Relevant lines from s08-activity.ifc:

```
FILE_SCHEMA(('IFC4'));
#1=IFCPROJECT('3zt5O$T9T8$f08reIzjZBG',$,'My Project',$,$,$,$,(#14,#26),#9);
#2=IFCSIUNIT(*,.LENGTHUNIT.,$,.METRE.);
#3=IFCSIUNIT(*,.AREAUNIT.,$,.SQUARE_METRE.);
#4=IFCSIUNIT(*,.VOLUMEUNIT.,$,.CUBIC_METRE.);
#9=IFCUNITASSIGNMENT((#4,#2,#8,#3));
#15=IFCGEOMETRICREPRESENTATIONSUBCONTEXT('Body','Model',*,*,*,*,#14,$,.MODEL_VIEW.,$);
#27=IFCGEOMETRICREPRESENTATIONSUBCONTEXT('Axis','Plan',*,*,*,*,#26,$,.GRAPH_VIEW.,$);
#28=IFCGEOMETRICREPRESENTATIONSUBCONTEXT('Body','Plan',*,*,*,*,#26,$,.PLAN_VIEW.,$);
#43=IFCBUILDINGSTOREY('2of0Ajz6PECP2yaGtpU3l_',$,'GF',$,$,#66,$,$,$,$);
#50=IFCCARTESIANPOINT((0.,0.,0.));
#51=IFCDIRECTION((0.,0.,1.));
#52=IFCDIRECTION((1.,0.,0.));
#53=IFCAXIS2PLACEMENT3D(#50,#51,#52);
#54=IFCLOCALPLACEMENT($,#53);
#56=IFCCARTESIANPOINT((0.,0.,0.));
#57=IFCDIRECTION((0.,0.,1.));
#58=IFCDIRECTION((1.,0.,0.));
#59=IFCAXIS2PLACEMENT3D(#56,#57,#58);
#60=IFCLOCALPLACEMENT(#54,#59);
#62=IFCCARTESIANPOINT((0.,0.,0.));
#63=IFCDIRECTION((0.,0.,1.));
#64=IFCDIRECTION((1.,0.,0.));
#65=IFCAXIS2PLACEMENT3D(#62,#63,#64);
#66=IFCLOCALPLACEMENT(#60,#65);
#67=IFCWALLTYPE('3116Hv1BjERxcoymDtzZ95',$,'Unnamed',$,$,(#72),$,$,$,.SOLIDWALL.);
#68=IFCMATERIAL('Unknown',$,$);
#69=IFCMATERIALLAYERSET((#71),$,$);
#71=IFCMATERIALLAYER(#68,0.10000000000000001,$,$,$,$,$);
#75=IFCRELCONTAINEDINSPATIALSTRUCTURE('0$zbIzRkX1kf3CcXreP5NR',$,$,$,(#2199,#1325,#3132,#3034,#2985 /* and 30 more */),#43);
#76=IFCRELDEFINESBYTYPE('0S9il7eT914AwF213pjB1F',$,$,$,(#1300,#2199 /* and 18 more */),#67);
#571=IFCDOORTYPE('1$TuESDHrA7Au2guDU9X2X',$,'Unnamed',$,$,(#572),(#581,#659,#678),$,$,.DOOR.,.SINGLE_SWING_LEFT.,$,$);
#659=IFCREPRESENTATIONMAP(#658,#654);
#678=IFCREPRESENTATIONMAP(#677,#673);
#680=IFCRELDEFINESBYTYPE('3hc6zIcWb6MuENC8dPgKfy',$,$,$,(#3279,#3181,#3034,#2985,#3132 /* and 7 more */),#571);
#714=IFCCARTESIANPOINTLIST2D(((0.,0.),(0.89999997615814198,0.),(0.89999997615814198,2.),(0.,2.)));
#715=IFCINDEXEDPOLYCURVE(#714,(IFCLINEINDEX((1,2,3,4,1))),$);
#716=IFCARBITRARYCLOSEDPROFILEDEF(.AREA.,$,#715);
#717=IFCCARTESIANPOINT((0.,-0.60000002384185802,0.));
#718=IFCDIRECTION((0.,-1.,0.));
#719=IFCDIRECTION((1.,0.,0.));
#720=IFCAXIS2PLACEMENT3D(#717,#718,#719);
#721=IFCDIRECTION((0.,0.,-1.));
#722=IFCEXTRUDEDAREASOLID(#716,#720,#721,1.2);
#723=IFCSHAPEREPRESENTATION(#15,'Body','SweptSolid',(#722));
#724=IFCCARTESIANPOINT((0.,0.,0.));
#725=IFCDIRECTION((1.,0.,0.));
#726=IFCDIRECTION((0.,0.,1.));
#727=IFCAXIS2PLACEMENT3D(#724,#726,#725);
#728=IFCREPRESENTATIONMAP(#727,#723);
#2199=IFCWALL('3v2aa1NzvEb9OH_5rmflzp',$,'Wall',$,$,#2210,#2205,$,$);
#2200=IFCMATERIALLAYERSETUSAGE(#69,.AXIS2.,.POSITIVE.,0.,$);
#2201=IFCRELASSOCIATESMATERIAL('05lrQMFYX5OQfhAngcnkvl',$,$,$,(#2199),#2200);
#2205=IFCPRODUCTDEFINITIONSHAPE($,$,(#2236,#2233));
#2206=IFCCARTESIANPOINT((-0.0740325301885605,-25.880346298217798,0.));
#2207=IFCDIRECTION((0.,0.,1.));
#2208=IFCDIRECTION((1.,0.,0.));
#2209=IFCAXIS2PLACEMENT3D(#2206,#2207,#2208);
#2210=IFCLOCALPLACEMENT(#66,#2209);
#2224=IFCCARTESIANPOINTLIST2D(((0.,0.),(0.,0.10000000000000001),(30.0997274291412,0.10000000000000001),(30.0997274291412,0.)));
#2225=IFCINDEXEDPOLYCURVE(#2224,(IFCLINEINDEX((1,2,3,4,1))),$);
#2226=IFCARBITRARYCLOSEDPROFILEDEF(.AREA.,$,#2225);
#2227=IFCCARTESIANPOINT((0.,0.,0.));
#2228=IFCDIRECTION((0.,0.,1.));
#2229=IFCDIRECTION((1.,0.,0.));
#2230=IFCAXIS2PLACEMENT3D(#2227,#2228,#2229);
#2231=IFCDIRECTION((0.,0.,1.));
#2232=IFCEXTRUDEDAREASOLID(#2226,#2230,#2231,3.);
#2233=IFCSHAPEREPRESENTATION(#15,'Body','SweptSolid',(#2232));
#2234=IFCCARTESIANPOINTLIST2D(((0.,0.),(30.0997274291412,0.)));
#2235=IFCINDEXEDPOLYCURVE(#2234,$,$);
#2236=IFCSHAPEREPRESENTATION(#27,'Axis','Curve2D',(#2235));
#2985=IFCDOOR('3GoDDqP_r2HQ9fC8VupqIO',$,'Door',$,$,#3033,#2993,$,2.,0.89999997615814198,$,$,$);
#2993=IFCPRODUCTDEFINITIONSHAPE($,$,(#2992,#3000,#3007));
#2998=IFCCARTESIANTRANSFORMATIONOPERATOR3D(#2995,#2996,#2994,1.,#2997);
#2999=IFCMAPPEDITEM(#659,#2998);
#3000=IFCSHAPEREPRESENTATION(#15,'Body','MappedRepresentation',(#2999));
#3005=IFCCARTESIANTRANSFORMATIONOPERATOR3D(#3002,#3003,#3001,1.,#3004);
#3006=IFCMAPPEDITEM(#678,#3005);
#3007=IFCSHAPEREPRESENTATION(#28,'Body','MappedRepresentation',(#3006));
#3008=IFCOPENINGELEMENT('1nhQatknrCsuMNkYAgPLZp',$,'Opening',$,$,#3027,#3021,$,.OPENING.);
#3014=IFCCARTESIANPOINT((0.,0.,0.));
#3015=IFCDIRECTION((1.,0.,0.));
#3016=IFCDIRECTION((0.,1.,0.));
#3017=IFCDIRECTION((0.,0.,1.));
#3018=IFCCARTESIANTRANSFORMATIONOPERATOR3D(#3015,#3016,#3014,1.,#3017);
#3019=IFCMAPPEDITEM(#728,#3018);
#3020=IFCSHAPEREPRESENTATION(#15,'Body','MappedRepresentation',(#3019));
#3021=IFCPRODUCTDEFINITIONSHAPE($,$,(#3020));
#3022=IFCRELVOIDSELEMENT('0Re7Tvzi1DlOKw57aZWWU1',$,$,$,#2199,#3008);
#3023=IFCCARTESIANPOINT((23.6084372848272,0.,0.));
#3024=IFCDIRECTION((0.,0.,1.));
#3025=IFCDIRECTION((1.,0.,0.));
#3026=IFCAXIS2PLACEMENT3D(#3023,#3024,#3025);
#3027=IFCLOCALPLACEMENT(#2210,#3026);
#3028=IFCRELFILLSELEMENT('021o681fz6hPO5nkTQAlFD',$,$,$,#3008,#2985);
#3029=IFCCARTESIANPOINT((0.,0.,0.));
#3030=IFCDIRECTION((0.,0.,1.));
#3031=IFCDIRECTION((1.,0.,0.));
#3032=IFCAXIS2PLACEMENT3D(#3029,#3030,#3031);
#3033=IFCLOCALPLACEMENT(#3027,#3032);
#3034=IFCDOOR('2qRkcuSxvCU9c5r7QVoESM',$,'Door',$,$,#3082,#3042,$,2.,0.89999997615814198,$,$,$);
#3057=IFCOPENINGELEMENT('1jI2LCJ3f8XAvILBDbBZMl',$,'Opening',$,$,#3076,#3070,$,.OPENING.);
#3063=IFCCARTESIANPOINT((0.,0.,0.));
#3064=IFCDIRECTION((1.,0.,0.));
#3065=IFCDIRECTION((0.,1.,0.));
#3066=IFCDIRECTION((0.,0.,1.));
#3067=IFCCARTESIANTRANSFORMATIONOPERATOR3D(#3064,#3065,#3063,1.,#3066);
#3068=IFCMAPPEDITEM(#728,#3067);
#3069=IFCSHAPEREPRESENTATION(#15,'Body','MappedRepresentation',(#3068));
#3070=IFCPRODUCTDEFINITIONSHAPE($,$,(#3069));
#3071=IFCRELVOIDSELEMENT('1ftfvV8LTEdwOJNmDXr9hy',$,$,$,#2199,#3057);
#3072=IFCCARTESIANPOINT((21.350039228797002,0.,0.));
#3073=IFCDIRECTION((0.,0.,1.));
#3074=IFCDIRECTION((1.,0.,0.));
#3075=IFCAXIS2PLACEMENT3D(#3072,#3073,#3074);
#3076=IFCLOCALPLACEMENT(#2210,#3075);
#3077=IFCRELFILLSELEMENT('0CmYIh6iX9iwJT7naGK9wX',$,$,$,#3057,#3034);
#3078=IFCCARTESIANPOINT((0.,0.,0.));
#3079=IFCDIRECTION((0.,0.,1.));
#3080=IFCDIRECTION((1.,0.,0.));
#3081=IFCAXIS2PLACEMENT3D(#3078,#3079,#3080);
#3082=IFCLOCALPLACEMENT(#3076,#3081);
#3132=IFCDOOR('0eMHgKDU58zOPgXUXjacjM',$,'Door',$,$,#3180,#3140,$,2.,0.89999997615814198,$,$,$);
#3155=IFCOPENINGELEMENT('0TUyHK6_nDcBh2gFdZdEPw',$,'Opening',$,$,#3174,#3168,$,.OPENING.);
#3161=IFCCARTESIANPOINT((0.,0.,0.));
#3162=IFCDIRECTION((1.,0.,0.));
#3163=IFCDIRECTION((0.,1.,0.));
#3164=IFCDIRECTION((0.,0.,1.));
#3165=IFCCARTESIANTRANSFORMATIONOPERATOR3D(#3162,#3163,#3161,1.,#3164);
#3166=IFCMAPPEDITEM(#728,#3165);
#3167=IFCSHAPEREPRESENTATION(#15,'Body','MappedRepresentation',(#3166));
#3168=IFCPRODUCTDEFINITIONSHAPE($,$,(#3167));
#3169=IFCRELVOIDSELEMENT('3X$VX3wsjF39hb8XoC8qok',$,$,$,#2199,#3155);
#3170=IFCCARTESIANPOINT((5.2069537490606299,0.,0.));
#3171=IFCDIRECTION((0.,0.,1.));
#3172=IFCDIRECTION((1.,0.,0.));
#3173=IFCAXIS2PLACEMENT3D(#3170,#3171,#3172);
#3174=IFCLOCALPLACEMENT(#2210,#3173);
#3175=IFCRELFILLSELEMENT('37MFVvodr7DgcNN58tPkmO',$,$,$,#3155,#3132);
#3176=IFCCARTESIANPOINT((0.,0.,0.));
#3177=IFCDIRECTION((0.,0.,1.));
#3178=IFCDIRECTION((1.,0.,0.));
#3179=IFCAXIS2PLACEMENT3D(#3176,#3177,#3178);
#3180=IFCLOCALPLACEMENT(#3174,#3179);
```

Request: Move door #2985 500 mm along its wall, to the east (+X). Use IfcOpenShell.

```python
import ifcopenshell
import ifcopenshell.api.geometry
import ifcopenshell.util.placement
import ifcopenshell.util.unit

model = ifcopenshell.open("s08-activity.ifc")
unit_scale = ifcopenshell.util.unit.calculate_unit_scale(model)

door = model.by_id(2985)
opening = door.FillsVoids[0].RelatingOpeningElement
wall = opening.VoidsElements[0].RelatingBuildingElement

wall_matrix = ifcopenshell.util.placement.get_local_placement(wall.ObjectPlacement)
shift = wall_matrix[:3, 0] * 0.5 / unit_scale
before = ifcopenshell.util.placement.get_local_placement(door.ObjectPlacement)[:3, 3].copy()

# The door is placed relative to its opening, so it follows when the opening moves.
matrix = ifcopenshell.util.placement.get_local_placement(opening.ObjectPlacement)
matrix[:3, 3] += shift
ifcopenshell.api.geometry.edit_object_placement(
    model, product=opening, matrix=matrix, is_si=False, should_transform_children=True
)

after = ifcopenshell.util.placement.get_local_placement(door.ObjectPlacement)[:3, 3]
print("door moved by", (after - before).round(3) + 0.0)

model.write("s08-activity_edited.ifc")
```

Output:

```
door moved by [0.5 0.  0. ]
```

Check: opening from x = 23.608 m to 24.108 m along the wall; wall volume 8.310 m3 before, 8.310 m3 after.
